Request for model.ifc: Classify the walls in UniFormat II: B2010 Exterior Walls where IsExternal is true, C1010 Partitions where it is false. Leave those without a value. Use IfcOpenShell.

First a look at what the model holds.

```python
import ifcopenshell
import ifcopenshell.util.element

model = ifcopenshell.open("model.ifc")
print(model.schema)
print("classifications:", [c.Name for c in model.by_type("IfcClassification")])
values = [ifcopenshell.util.element.get_pset(e, "Pset_WallCommon", "IsExternal") for e in model.by_type("IfcWall")]
for value in (True, False, None):
    print("IsExternal", value, values.count(value))
```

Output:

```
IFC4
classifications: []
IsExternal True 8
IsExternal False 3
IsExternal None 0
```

```python
import ifcopenshell
import ifcopenshell.api.classification
import ifcopenshell.util.element

model = ifcopenshell.open("model.ifc")

system = ifcopenshell.api.classification.add_classification(model, classification="UniFormat II")

walls = model.by_type("IfcWall")
external = {e: ifcopenshell.util.element.get_pset(e, "Pset_WallCommon", "IsExternal") for e in walls}
for flag, code, name in ((True, "B2010", "Exterior Walls"), (False, "C1010", "Partitions")):
    products = [e for e in walls if external[e] is flag]
    ifcopenshell.api.classification.add_reference(
        model, products=products, classification=system, identification=code, name=name
    )
    print(code, len(products))

model.write("model_v2.ifc")
```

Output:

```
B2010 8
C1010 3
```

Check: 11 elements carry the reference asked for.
